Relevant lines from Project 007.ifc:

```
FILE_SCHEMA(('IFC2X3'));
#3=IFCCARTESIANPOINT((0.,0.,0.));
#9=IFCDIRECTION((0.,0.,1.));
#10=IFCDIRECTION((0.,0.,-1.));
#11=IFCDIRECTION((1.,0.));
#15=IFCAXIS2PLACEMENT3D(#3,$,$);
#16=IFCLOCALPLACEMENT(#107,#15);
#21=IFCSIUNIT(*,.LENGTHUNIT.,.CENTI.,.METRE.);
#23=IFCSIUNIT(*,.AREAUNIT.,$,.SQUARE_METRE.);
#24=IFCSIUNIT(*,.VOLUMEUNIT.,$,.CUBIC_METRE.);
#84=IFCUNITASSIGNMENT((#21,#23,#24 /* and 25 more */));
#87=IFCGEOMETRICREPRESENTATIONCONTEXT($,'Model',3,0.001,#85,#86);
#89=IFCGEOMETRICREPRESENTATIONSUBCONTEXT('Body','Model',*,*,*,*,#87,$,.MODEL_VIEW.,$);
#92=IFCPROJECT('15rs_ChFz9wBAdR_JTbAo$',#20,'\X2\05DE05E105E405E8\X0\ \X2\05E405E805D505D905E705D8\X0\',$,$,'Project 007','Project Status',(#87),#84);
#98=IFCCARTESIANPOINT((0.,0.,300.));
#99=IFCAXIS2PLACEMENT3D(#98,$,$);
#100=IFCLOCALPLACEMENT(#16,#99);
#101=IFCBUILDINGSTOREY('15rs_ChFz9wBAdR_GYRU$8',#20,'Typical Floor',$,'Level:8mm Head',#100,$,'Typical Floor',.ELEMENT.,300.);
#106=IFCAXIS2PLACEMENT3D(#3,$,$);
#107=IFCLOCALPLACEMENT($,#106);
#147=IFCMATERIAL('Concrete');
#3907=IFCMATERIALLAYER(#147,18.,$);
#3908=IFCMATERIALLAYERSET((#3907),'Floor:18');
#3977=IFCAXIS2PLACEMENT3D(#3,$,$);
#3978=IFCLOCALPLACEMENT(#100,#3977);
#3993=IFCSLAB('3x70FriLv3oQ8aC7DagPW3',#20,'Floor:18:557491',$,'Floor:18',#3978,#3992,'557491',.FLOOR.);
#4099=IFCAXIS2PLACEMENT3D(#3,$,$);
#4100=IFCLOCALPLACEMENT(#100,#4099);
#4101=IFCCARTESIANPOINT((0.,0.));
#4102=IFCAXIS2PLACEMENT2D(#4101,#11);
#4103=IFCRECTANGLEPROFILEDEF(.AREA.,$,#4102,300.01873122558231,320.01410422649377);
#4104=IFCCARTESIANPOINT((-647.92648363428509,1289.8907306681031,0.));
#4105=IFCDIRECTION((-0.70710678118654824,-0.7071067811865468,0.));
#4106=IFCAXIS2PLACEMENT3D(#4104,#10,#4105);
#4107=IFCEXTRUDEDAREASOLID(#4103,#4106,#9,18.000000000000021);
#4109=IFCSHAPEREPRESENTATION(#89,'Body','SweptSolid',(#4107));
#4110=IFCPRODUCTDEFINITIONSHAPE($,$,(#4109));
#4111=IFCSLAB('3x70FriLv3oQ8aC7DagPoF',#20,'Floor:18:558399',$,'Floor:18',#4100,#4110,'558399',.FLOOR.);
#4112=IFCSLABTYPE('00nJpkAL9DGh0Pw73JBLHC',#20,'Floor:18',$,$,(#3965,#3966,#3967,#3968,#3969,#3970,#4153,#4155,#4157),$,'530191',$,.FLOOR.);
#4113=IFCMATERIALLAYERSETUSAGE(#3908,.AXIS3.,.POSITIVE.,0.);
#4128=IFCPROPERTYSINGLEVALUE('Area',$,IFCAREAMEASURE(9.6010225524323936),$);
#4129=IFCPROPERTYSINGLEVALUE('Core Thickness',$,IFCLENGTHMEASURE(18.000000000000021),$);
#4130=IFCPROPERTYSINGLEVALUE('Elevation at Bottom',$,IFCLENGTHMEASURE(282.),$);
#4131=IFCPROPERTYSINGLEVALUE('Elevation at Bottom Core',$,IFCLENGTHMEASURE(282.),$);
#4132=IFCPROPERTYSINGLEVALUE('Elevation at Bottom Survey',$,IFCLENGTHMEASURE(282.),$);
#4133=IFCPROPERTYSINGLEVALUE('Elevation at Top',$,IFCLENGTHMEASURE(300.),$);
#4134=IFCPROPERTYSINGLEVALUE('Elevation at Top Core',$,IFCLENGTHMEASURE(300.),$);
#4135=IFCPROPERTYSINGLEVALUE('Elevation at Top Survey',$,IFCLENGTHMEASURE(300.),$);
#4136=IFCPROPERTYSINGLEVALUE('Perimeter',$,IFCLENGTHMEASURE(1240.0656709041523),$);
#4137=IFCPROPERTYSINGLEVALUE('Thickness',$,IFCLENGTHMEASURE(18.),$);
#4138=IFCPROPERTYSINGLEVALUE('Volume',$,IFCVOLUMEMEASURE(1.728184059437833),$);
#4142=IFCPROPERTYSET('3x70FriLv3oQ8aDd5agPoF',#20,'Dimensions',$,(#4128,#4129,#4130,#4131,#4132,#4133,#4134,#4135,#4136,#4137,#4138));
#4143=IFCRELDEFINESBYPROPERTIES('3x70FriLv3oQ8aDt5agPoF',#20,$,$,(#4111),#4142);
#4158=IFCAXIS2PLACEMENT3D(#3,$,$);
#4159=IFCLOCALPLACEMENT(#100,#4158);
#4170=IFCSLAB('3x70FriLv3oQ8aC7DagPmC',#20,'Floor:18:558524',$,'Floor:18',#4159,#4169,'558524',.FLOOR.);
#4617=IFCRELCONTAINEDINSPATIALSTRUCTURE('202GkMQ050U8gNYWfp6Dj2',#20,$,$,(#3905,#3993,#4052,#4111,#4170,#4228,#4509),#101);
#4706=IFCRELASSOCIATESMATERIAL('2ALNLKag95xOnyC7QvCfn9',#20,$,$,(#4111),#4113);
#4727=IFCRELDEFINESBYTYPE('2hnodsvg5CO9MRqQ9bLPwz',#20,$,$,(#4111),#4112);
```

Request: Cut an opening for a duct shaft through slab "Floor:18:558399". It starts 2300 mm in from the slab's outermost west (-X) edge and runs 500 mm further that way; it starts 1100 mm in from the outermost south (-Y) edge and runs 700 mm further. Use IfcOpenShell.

```python
import numpy as np
import ifcopenshell
import ifcopenshell.api.feature
import ifcopenshell.api.geometry
import ifcopenshell.api.pset
import ifcopenshell.api.root
import ifcopenshell.geom
import ifcopenshell.util.element
import ifcopenshell.util.placement
import ifcopenshell.util.representation
import ifcopenshell.util.shape
import ifcopenshell.util.unit

model = ifcopenshell.open("Project 007.ifc")
unit_scale = ifcopenshell.util.unit.calculate_unit_scale(model)
area_scale = ifcopenshell.util.unit.calculate_unit_scale(model, "AREAUNIT")
volume_scale = ifcopenshell.util.unit.calculate_unit_scale(model, "VOLUMEUNIT")
settings = ifcopenshell.geom.settings()


def volume(element):
    """Net volume in cubic metres, openings subtracted."""
    shape = ifcopenshell.geom.create_shape(settings, element)
    return ifcopenshell.util.shape.get_volume(shape.geometry)


slab = model.by_guid("3x70FriLv3oQ8aC7DagPoF")
before = volume(slab)

# Extent in the slab's own axes, in metres. The edges named are its -X and -Y sides.
slab_shape = ifcopenshell.geom.create_shape(settings, slab)
vertices = ifcopenshell.util.shape.get_vertices(slab_shape.geometry)
x_min, y_min, bottom = vertices.min(axis=0)
top = vertices[:, 2].max()

opening = ifcopenshell.api.root.create_entity(model, ifc_class="IfcOpeningElement", name="Duct shaft opening")
context = ifcopenshell.util.representation.get_context(model, "Model", "Body", "MODEL_VIEW")
width, depth = 0.5, 0.7
outline = [(0.0, 0.0), (width, 0.0), (width, depth), (0.0, depth), (0.0, 0.0)]
# Overshoot both faces by 50 mm so the cut is clean.
shape = ifcopenshell.api.geometry.add_slab_representation(
    model, context=context, depth=top - bottom + 0.1, polyline=outline
)
ifcopenshell.api.geometry.assign_representation(model, product=opening, representation=shape)

matrix = ifcopenshell.util.placement.get_local_placement(slab.ObjectPlacement)
matrix[:, 3] = matrix @ np.append(np.array([x_min + 2.3, y_min + 1.1, bottom - 0.05]) / unit_scale, 1.0)
ifcopenshell.api.geometry.edit_object_placement(model, product=opening, matrix=matrix, is_si=False)
ifcopenshell.api.feature.add_feature(model, feature=opening, element=slab)

after = volume(slab)

# Update the slab's stored quantities.
pset = model.by_id(ifcopenshell.util.element.get_pset(slab, "Dimensions", should_inherit=False)["id"])
ifcopenshell.api.pset.edit_pset(model, pset=pset, properties={
    "Area": model.create_entity("IfcAreaMeasure", after / (top - bottom) / area_scale),
    "Volume": model.create_entity("IfcVolumeMeasure", after / volume_scale),
})

print(f"slab volume {before:.3f} -> {after:.3f} m3")

model.write("Project 007_updated.ifc")
```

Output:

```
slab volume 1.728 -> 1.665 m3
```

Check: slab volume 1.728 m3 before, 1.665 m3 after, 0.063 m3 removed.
